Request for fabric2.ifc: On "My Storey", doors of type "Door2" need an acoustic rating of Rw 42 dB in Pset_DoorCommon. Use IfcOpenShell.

First a look at what the model holds.

```python
import ifcopenshell
import ifcopenshell.util.element

model = ifcopenshell.open("fabric2.ifc")
print(model.schema)
storey = next(s for s in model.by_type("IfcBuildingStorey") if s.Name == "My Storey")
doors = [e for e in ifcopenshell.util.element.get_decomposition(storey) if e.is_a("IfcDoor")]
seen = {}
for e in doors:
    element_type = ifcopenshell.util.element.get_type(e)
    key = (element_type.Name if element_type != e and element_type else None, ifcopenshell.util.element.get_pset(e, "Pset_DoorCommon", "AcousticRating"))
    seen[key] = seen.get(key, 0) + 1
for (name, value), count in sorted(seen.items(), key=str):
    print(count, "x", name, "|", value)
```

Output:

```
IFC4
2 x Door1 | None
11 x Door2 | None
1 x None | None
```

```python
import ifcopenshell
import ifcopenshell.api.pset
import ifcopenshell.util.element

model = ifcopenshell.open("fabric2.ifc")

storey = next(s for s in model.by_type("IfcBuildingStorey") if s.Name == "My Storey")
doors = [e for e in ifcopenshell.util.element.get_decomposition(storey) if e.is_a("IfcDoor")]

count = 0
for e in doors:
    element_type = ifcopenshell.util.element.get_type(e)
    if element_type in (None, e) or element_type.Name != "Door2":
        continue
    # add_pset returns the element's existing set when there is one.
    pset = ifcopenshell.api.pset.add_pset(model, product=e, name="Pset_DoorCommon")
    ifcopenshell.api.pset.edit_pset(model, pset=pset, properties={"AcousticRating": "Rw 42 dB"})
    count += 1

print(count, "doors updated")

model.write("fabric2_rev.ifc")
```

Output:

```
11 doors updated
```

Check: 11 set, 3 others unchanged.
